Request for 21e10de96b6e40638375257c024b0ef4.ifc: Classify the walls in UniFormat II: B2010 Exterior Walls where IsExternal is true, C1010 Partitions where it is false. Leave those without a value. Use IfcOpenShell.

First a look at what the model holds.

```python
import ifcopenshell
import ifcopenshell.util.element

model = ifcopenshell.open("21e10de96b6e40638375257c024b0ef4.ifc")
print(model.schema)
print("classifications:", [c.Name for c in model.by_type("IfcClassification")])
values = [ifcopenshell.util.element.get_pset(e, "Pset_WallCommon", "IsExternal") for e in model.by_type("IfcWall")]
for value in (True, False, None):
    print("IsExternal", value, values.count(value))
```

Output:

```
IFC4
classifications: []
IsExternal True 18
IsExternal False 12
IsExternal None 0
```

```python
import ifcopenshell
import ifcopenshell.api.classification
import ifcopenshell.util.element

model = ifcopenshell.open("21e10de96b6e40638375257c024b0ef4.ifc")

system = ifcopenshell.api.classification.add_classification(model, classification="UniFormat II")

walls = model.by_type("IfcWall")
external = {e: ifcopenshell.util.element.get_pset(e, "Pset_WallCommon", "IsExternal") for e in walls}
for flag, code, name in ((True, "B2010", "Exterior Walls"), (False, "C1010", "Partitions")):
    products = [e for e in walls if external[e] is flag]
    ifcopenshell.api.classification.add_reference(
        model, products=products, classification=system, identification=code, name=name
    )
    print(code, len(products))

model.write("21e10de96b6e40638375257c024b0ef4_edited.ifc")
```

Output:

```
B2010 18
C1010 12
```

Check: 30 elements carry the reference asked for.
